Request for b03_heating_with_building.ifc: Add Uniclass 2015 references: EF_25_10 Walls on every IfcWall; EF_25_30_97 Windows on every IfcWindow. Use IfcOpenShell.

First a look at what the model holds.

```python
import ifcopenshell

model = ifcopenshell.open("b03_heating_with_building.ifc")
print(model.schema)
print("classifications:", [c.Name for c in model.by_type("IfcClassification")])
for ifc_class in ("IfcDoor", "IfcRoof", "IfcStair", "IfcWall", "IfcWindow"):
    print(ifc_class, len(model.by_type(ifc_class)))
```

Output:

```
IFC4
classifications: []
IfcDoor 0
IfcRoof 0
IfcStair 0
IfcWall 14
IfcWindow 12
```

```python
import ifcopenshell
import ifcopenshell.api.classification

model = ifcopenshell.open("b03_heating_with_building.ifc")

system = ifcopenshell.api.classification.add_classification(model, classification="Uniclass 2015")

codes = {
    "IfcWall": ("EF_25_10", "Walls"),
    "IfcWindow": ("EF_25_30_97", "Windows"),
}
for ifc_class, (code, name) in codes.items():
    products = model.by_type(ifc_class)
    ifcopenshell.api.classification.add_reference(
        model, products=products, classification=system, identification=code, name=name
    )
    print(code, len(products))

model.write("b03_heating_with_building_updated.ifc")
```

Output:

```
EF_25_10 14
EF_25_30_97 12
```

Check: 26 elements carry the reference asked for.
